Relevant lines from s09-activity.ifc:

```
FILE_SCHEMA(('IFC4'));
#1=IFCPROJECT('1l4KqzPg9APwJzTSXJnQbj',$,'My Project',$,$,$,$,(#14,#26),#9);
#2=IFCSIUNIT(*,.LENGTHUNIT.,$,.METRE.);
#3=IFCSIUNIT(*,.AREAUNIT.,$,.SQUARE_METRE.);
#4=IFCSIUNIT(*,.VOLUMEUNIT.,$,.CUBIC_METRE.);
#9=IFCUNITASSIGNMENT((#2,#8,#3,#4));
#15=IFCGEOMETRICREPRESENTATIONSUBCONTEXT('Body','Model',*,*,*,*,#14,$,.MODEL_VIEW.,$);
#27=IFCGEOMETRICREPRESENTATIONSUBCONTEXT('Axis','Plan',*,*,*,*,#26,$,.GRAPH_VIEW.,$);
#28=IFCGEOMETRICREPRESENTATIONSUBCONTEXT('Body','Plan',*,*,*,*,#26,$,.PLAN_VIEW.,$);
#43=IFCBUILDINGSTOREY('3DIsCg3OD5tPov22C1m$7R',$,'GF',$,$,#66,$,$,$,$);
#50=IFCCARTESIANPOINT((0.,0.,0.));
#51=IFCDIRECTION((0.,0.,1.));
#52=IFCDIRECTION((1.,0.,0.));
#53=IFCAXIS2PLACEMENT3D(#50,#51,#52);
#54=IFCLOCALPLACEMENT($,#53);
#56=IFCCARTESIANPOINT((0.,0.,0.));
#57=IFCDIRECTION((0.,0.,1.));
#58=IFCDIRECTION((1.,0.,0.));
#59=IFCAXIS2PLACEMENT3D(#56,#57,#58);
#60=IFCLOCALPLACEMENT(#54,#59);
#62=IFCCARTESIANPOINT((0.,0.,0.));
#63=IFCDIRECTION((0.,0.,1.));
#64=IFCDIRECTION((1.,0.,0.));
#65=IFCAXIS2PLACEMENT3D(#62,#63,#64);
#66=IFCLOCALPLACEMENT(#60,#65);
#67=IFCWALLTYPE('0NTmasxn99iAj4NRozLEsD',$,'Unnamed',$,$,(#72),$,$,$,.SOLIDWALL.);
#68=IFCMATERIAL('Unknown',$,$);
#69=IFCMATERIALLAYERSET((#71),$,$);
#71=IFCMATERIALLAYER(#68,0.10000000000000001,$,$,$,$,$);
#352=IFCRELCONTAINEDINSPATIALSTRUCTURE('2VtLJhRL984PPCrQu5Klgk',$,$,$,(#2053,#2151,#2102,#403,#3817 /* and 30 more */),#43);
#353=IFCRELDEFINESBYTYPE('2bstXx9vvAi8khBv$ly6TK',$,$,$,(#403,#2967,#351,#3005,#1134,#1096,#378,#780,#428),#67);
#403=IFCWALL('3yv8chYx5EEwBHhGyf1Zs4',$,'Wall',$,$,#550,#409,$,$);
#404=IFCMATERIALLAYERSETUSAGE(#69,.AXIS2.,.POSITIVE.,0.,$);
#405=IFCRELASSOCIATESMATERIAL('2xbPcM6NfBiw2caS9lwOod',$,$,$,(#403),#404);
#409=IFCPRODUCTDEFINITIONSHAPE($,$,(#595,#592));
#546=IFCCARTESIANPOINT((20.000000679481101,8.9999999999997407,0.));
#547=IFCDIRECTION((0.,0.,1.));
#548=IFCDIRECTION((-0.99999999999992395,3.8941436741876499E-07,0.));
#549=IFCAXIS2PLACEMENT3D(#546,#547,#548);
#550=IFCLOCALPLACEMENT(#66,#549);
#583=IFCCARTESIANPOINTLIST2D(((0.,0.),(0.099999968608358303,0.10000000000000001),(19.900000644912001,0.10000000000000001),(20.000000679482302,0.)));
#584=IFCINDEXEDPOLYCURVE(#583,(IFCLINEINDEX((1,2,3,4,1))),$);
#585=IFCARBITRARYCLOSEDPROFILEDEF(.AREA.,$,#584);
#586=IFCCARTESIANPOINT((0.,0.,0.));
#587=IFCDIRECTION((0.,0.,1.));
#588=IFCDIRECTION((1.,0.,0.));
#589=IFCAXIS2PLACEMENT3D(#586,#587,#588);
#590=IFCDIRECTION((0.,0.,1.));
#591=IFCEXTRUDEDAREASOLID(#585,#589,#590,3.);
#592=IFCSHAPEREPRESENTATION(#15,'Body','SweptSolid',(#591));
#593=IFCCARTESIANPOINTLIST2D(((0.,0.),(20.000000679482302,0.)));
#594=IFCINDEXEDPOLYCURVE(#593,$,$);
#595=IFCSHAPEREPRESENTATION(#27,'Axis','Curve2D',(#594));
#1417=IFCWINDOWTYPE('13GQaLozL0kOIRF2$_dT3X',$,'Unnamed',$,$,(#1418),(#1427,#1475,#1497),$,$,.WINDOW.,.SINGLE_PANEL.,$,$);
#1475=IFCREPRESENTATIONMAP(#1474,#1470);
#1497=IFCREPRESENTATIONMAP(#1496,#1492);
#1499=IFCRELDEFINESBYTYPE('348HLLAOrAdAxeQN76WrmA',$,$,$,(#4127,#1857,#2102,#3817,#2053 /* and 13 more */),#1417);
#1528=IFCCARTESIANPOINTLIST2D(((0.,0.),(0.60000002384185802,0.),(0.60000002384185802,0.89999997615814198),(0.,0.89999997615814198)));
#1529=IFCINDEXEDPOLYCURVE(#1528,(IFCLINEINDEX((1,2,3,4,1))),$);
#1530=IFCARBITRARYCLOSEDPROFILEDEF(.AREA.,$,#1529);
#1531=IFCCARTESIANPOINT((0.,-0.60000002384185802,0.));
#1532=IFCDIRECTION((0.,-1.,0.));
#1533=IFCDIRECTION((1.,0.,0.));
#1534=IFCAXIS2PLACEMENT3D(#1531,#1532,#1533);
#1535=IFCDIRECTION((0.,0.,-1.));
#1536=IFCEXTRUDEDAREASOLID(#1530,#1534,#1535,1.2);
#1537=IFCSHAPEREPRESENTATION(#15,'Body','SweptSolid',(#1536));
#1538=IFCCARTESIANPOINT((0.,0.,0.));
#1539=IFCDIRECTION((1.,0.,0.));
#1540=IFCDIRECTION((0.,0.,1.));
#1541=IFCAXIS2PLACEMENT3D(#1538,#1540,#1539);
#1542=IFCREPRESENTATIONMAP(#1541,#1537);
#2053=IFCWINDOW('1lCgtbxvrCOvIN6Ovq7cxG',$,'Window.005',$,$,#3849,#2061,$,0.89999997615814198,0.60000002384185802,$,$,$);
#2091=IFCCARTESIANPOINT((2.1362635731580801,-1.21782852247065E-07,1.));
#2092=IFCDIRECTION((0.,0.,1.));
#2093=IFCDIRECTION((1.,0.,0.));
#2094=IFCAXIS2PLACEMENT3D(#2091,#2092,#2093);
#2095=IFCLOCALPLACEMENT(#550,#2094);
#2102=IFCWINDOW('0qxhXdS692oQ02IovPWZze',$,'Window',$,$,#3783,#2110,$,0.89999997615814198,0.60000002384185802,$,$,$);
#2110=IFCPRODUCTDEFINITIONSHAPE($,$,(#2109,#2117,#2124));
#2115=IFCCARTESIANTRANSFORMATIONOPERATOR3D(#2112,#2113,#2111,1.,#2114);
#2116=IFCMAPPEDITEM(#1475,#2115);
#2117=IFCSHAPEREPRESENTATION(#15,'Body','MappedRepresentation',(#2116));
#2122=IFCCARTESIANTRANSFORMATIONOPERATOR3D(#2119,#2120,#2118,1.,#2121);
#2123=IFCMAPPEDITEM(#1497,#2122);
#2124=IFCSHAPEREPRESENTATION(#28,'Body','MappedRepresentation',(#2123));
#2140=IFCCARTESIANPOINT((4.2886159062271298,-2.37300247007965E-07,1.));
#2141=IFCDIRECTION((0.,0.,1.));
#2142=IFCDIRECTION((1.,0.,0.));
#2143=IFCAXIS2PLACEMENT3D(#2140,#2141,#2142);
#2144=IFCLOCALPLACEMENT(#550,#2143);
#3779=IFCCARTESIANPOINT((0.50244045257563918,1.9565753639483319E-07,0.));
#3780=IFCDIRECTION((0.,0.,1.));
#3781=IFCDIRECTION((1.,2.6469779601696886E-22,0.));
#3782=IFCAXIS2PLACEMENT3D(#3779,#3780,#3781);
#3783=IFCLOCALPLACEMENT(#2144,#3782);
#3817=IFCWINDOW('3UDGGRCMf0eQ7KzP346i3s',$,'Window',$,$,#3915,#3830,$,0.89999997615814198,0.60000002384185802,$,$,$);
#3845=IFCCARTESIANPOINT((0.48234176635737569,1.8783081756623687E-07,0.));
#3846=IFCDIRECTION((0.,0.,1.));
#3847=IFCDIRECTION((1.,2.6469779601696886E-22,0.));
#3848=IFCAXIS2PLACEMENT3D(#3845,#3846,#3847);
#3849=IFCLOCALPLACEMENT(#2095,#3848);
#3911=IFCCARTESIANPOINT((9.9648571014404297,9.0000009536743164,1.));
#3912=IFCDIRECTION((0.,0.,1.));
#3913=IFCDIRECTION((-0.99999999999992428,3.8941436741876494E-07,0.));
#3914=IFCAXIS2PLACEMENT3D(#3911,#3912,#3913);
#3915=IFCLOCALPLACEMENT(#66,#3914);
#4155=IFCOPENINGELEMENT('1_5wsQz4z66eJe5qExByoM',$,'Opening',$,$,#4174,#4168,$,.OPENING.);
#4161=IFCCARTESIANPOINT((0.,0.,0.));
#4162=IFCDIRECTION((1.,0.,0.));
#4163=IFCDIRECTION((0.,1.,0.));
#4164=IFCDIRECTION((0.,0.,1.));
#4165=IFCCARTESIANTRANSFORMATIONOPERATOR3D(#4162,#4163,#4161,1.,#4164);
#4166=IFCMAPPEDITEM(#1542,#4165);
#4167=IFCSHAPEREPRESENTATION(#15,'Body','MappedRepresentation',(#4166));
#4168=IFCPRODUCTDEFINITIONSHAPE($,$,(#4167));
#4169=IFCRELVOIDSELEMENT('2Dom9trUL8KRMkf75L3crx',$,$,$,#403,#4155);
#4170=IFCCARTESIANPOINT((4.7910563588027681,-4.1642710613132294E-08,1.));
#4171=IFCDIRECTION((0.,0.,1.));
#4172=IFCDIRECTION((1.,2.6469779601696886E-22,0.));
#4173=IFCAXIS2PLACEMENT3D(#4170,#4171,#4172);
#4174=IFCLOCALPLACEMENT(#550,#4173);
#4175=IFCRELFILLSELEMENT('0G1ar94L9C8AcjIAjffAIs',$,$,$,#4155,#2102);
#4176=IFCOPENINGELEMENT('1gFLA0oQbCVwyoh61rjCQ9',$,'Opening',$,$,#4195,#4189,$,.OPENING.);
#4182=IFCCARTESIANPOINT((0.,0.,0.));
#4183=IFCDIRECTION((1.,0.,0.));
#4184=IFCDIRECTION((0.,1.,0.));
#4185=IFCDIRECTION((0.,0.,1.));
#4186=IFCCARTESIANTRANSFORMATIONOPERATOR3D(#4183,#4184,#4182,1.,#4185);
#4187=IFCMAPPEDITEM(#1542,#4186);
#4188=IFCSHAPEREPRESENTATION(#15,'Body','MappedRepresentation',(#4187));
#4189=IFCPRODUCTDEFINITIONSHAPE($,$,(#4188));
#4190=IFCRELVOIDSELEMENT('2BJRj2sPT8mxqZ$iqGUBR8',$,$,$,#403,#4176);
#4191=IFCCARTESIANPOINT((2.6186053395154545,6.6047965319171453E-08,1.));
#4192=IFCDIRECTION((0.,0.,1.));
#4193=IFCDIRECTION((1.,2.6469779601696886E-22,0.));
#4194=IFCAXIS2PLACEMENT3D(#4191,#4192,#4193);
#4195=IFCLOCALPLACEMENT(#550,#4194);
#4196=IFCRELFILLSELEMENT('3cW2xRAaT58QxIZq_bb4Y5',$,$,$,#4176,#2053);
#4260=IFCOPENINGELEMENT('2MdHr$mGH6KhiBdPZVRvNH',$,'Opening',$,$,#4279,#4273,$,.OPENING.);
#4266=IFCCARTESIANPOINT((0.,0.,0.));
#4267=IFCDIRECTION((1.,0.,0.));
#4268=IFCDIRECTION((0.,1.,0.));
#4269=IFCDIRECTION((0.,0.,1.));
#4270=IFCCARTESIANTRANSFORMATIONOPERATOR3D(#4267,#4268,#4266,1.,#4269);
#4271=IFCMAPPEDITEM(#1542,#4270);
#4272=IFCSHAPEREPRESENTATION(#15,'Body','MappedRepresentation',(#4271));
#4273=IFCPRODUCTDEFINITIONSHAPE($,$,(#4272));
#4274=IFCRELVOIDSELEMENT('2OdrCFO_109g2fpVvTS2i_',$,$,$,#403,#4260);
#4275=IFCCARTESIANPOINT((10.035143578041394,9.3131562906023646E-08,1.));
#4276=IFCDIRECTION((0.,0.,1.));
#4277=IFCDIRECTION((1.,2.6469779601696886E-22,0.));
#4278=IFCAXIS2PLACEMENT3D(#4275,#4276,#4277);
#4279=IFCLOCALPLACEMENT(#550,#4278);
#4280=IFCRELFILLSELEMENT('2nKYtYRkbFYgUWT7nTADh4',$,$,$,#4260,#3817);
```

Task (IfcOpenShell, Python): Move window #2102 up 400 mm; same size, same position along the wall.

```python
import numpy as np
import ifcopenshell
import ifcopenshell.api.geometry
import ifcopenshell.util.placement
import ifcopenshell.util.unit

model = ifcopenshell.open("s09-activity.ifc")
unit_scale = ifcopenshell.util.unit.calculate_unit_scale(model)

window = model.by_guid("0qxhXdS692oQ02IovPWZze")
opening = window.FillsVoids[0].RelatingOpeningElement
dz = 0.4

shift = np.array([0.0, 0.0, dz])
# The window is not placed relative to its opening, so move both.
for product in (opening, window):
    matrix = ifcopenshell.util.placement.get_local_placement(product.ObjectPlacement)
    matrix[:3, 3] += shift
    ifcopenshell.api.geometry.edit_object_placement(model, product=product, matrix=matrix, is_si=False)

print(f"moved by {dz * unit_scale:+.3f} m")

model.write("s09-activity_rev.ifc")
```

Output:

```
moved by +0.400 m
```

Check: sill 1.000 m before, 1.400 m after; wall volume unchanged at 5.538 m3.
